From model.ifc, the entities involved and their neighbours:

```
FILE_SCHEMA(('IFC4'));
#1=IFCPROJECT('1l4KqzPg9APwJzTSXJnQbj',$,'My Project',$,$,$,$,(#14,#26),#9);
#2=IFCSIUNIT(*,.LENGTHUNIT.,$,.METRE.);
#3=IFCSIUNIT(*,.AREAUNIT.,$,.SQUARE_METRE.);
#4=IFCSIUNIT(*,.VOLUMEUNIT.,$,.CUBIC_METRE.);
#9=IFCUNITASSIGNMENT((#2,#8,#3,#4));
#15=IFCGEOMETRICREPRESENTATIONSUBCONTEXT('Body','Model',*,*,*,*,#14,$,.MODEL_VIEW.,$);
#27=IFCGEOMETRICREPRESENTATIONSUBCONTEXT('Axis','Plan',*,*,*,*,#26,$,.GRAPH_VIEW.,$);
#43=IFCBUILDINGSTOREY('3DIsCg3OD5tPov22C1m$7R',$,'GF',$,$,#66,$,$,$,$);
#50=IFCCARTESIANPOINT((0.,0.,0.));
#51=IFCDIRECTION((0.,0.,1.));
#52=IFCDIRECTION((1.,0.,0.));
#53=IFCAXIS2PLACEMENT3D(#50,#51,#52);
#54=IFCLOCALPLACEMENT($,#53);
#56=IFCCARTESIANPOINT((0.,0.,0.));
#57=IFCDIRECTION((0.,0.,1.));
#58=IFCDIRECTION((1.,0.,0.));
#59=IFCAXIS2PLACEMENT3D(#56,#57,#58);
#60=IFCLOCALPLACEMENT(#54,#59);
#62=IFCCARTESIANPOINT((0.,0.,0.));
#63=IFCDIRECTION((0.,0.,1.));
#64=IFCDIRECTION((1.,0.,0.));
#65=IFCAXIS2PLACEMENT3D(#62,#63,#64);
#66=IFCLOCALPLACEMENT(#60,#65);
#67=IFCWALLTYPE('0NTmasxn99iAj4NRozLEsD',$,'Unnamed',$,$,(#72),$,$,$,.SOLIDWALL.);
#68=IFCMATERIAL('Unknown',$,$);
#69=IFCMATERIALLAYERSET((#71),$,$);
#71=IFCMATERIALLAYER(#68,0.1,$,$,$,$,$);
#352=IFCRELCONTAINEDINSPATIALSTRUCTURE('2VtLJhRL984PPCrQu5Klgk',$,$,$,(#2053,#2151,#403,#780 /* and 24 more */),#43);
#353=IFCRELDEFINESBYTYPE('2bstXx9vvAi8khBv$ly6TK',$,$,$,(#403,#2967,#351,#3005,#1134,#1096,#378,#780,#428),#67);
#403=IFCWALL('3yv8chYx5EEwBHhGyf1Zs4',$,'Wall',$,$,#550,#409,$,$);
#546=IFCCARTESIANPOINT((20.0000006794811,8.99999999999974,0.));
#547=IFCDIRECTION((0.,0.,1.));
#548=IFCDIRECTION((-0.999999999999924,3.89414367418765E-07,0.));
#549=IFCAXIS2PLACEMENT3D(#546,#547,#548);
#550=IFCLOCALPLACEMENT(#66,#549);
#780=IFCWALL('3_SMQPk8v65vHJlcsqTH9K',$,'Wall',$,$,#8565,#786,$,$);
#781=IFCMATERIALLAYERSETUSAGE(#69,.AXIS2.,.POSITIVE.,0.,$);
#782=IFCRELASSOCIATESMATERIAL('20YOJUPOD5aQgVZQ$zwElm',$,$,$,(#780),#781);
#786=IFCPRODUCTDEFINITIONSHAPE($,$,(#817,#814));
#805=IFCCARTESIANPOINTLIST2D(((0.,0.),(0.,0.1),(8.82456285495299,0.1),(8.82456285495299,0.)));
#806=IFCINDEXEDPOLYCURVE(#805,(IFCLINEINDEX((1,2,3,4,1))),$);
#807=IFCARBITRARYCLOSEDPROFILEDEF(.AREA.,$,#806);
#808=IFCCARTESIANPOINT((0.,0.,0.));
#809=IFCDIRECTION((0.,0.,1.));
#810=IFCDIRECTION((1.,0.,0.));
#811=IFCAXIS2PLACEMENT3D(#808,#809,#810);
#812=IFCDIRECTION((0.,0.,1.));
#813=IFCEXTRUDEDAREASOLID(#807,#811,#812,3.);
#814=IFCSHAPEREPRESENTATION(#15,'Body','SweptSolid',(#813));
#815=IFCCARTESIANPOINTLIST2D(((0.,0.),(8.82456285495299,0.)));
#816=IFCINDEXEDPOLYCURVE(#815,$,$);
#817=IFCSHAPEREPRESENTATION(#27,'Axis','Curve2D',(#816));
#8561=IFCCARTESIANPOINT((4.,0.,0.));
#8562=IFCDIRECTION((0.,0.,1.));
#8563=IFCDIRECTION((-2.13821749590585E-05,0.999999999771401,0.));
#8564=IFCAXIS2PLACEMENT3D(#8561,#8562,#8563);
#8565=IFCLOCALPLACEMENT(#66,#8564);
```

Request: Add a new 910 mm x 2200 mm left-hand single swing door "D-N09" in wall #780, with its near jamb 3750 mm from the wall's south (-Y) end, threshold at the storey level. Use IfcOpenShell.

```python
import numpy as np
import ifcopenshell
import ifcopenshell.api.feature
import ifcopenshell.api.geometry
import ifcopenshell.api.root
import ifcopenshell.api.spatial
import ifcopenshell.geom
import ifcopenshell.util.element
import ifcopenshell.util.placement
import ifcopenshell.util.representation
import ifcopenshell.util.shape
import ifcopenshell.util.unit

model = ifcopenshell.open("model.ifc")
unit_scale = ifcopenshell.util.unit.calculate_unit_scale(model)
settings = ifcopenshell.geom.settings()


def volume(element):
    """Net volume in cubic metres, openings subtracted."""
    shape = ifcopenshell.geom.create_shape(settings, element)
    return ifcopenshell.util.shape.get_volume(shape.geometry)


wall = model.by_guid("3_SMQPk8v65vHJlcsqTH9K")
storey = ifcopenshell.util.element.get_container(wall, ifc_class="IfcBuildingStorey")
context = ifcopenshell.util.representation.get_context(model, "Model", "Body", "MODEL_VIEW")
before = volume(wall)

width, height, from_end, sill = 0.91, 2.2, 3.75, 0.0  # metres

# The wall runs along its own X axis, and the end named is its -X end.
wall_shape = ifcopenshell.geom.create_shape(settings, wall)
x, y, z = ifcopenshell.util.shape.get_vertices(wall_shape.geometry).T
start = x.min() + from_end
face, thickness = float(y.min()), float(y.max() - y.min())
wall_matrix = ifcopenshell.util.placement.get_local_placement(wall.ObjectPlacement)
level = ifcopenshell.util.placement.get_local_placement(storey.ObjectPlacement)[2, 3]


def in_wall(x, y):
    """Placement at x, y metres in the wall's axes, at sill height."""
    matrix = wall_matrix.copy()
    matrix[:, 3] = wall_matrix @ np.array([x / unit_scale, y / unit_scale, 0.0, 1.0])
    matrix[2, 3] = level + sill / unit_scale
    return matrix


# Opening: a box that overshoots both wall faces by 50 mm.
opening = ifcopenshell.api.root.create_entity(model, ifc_class="IfcOpeningElement", predefined_type="OPENING")
box = ifcopenshell.api.geometry.add_wall_representation(
    model, context=context, length=width, height=height, thickness=thickness + 0.1
)
ifcopenshell.api.geometry.assign_representation(model, product=opening, representation=box)
ifcopenshell.api.geometry.edit_object_placement(model, product=opening, matrix=in_wall(start, face - 0.05), is_si=False)
ifcopenshell.api.feature.add_feature(model, feature=opening, element=wall)

door = ifcopenshell.api.root.create_entity(model, ifc_class="IfcDoor", name="D-N09", predefined_type="DOOR")
door.OverallWidth, door.OverallHeight = width / unit_scale, height / unit_scale
door.OperationType = "SINGLE_SWING_LEFT"
body = ifcopenshell.api.geometry.add_door_representation(
    model,
    context=context,
    overall_width=door.OverallWidth,
    overall_height=door.OverallHeight,
    operation_type="SINGLE_SWING_LEFT",
    lining_properties={"LiningDepth": thickness / unit_scale, "ThresholdDepth": thickness / unit_scale},
)
ifcopenshell.api.geometry.assign_representation(model, product=door, representation=body)
ifcopenshell.api.spatial.assign_container(model, products=[door], relating_structure=storey)
ifcopenshell.api.feature.add_filling(model, opening=opening, element=door)

# The lining spans the wall, so the door starts at the wall face.
ifcopenshell.api.geometry.edit_object_placement(model, product=door, matrix=in_wall(start, face), is_si=False)

after = volume(wall)

print(f"wall volume {before:.3f} -> {after:.3f} m3")

model.write("model-out.ifc")
```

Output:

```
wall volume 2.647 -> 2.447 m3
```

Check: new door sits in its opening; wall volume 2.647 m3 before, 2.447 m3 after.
